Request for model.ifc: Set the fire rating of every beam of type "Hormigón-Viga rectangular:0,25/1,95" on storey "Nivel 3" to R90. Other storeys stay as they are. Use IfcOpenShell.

First a look at what the model holds.

```python
import ifcopenshell
import ifcopenshell.util.element

model = ifcopenshell.open("model.ifc")
print(model.schema)
storey = next(s for s in model.by_type("IfcBuildingStorey") if s.Name == "Nivel 3")
beams = [e for e in ifcopenshell.util.element.get_decomposition(storey) if e.is_a("IfcBeam")]
seen = {}
for e in beams:
    element_type = ifcopenshell.util.element.get_type(e)
    key = (element_type.Name if element_type != e and element_type else None, ifcopenshell.util.element.get_pset(e, "Pset_BeamCommon", "FireRating"))
    seen[key] = seen.get(key, 0) + 1
for (name, value), count in sorted(seen.items(), key=str):
    print(count, "x", name, "|", value)
```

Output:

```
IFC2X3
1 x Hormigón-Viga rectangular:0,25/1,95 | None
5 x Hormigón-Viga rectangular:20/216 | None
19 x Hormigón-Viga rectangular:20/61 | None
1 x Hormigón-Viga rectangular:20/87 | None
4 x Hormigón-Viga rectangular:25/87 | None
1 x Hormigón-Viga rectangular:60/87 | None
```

```python
import ifcopenshell
import ifcopenshell.api.pset
import ifcopenshell.util.element

model = ifcopenshell.open("model.ifc")

storey = next(s for s in model.by_type("IfcBuildingStorey") if s.Name == "Nivel 3")
beams = [e for e in ifcopenshell.util.element.get_decomposition(storey) if e.is_a("IfcBeam")]

count = 0
for e in beams:
    element_type = ifcopenshell.util.element.get_type(e)
    if element_type in (None, e) or element_type.Name != "Hormigón-Viga rectangular:0,25/1,95":
        continue
    # add_pset returns the element's existing set when there is one.
    pset = ifcopenshell.api.pset.add_pset(model, product=e, name="Pset_BeamCommon")
    ifcopenshell.api.pset.edit_pset(model, pset=pset, properties={"FireRating": "R90"})
    count += 1

print(count, "beams updated")

model.write("model_v2.ifc")
```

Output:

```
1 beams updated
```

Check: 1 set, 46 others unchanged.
